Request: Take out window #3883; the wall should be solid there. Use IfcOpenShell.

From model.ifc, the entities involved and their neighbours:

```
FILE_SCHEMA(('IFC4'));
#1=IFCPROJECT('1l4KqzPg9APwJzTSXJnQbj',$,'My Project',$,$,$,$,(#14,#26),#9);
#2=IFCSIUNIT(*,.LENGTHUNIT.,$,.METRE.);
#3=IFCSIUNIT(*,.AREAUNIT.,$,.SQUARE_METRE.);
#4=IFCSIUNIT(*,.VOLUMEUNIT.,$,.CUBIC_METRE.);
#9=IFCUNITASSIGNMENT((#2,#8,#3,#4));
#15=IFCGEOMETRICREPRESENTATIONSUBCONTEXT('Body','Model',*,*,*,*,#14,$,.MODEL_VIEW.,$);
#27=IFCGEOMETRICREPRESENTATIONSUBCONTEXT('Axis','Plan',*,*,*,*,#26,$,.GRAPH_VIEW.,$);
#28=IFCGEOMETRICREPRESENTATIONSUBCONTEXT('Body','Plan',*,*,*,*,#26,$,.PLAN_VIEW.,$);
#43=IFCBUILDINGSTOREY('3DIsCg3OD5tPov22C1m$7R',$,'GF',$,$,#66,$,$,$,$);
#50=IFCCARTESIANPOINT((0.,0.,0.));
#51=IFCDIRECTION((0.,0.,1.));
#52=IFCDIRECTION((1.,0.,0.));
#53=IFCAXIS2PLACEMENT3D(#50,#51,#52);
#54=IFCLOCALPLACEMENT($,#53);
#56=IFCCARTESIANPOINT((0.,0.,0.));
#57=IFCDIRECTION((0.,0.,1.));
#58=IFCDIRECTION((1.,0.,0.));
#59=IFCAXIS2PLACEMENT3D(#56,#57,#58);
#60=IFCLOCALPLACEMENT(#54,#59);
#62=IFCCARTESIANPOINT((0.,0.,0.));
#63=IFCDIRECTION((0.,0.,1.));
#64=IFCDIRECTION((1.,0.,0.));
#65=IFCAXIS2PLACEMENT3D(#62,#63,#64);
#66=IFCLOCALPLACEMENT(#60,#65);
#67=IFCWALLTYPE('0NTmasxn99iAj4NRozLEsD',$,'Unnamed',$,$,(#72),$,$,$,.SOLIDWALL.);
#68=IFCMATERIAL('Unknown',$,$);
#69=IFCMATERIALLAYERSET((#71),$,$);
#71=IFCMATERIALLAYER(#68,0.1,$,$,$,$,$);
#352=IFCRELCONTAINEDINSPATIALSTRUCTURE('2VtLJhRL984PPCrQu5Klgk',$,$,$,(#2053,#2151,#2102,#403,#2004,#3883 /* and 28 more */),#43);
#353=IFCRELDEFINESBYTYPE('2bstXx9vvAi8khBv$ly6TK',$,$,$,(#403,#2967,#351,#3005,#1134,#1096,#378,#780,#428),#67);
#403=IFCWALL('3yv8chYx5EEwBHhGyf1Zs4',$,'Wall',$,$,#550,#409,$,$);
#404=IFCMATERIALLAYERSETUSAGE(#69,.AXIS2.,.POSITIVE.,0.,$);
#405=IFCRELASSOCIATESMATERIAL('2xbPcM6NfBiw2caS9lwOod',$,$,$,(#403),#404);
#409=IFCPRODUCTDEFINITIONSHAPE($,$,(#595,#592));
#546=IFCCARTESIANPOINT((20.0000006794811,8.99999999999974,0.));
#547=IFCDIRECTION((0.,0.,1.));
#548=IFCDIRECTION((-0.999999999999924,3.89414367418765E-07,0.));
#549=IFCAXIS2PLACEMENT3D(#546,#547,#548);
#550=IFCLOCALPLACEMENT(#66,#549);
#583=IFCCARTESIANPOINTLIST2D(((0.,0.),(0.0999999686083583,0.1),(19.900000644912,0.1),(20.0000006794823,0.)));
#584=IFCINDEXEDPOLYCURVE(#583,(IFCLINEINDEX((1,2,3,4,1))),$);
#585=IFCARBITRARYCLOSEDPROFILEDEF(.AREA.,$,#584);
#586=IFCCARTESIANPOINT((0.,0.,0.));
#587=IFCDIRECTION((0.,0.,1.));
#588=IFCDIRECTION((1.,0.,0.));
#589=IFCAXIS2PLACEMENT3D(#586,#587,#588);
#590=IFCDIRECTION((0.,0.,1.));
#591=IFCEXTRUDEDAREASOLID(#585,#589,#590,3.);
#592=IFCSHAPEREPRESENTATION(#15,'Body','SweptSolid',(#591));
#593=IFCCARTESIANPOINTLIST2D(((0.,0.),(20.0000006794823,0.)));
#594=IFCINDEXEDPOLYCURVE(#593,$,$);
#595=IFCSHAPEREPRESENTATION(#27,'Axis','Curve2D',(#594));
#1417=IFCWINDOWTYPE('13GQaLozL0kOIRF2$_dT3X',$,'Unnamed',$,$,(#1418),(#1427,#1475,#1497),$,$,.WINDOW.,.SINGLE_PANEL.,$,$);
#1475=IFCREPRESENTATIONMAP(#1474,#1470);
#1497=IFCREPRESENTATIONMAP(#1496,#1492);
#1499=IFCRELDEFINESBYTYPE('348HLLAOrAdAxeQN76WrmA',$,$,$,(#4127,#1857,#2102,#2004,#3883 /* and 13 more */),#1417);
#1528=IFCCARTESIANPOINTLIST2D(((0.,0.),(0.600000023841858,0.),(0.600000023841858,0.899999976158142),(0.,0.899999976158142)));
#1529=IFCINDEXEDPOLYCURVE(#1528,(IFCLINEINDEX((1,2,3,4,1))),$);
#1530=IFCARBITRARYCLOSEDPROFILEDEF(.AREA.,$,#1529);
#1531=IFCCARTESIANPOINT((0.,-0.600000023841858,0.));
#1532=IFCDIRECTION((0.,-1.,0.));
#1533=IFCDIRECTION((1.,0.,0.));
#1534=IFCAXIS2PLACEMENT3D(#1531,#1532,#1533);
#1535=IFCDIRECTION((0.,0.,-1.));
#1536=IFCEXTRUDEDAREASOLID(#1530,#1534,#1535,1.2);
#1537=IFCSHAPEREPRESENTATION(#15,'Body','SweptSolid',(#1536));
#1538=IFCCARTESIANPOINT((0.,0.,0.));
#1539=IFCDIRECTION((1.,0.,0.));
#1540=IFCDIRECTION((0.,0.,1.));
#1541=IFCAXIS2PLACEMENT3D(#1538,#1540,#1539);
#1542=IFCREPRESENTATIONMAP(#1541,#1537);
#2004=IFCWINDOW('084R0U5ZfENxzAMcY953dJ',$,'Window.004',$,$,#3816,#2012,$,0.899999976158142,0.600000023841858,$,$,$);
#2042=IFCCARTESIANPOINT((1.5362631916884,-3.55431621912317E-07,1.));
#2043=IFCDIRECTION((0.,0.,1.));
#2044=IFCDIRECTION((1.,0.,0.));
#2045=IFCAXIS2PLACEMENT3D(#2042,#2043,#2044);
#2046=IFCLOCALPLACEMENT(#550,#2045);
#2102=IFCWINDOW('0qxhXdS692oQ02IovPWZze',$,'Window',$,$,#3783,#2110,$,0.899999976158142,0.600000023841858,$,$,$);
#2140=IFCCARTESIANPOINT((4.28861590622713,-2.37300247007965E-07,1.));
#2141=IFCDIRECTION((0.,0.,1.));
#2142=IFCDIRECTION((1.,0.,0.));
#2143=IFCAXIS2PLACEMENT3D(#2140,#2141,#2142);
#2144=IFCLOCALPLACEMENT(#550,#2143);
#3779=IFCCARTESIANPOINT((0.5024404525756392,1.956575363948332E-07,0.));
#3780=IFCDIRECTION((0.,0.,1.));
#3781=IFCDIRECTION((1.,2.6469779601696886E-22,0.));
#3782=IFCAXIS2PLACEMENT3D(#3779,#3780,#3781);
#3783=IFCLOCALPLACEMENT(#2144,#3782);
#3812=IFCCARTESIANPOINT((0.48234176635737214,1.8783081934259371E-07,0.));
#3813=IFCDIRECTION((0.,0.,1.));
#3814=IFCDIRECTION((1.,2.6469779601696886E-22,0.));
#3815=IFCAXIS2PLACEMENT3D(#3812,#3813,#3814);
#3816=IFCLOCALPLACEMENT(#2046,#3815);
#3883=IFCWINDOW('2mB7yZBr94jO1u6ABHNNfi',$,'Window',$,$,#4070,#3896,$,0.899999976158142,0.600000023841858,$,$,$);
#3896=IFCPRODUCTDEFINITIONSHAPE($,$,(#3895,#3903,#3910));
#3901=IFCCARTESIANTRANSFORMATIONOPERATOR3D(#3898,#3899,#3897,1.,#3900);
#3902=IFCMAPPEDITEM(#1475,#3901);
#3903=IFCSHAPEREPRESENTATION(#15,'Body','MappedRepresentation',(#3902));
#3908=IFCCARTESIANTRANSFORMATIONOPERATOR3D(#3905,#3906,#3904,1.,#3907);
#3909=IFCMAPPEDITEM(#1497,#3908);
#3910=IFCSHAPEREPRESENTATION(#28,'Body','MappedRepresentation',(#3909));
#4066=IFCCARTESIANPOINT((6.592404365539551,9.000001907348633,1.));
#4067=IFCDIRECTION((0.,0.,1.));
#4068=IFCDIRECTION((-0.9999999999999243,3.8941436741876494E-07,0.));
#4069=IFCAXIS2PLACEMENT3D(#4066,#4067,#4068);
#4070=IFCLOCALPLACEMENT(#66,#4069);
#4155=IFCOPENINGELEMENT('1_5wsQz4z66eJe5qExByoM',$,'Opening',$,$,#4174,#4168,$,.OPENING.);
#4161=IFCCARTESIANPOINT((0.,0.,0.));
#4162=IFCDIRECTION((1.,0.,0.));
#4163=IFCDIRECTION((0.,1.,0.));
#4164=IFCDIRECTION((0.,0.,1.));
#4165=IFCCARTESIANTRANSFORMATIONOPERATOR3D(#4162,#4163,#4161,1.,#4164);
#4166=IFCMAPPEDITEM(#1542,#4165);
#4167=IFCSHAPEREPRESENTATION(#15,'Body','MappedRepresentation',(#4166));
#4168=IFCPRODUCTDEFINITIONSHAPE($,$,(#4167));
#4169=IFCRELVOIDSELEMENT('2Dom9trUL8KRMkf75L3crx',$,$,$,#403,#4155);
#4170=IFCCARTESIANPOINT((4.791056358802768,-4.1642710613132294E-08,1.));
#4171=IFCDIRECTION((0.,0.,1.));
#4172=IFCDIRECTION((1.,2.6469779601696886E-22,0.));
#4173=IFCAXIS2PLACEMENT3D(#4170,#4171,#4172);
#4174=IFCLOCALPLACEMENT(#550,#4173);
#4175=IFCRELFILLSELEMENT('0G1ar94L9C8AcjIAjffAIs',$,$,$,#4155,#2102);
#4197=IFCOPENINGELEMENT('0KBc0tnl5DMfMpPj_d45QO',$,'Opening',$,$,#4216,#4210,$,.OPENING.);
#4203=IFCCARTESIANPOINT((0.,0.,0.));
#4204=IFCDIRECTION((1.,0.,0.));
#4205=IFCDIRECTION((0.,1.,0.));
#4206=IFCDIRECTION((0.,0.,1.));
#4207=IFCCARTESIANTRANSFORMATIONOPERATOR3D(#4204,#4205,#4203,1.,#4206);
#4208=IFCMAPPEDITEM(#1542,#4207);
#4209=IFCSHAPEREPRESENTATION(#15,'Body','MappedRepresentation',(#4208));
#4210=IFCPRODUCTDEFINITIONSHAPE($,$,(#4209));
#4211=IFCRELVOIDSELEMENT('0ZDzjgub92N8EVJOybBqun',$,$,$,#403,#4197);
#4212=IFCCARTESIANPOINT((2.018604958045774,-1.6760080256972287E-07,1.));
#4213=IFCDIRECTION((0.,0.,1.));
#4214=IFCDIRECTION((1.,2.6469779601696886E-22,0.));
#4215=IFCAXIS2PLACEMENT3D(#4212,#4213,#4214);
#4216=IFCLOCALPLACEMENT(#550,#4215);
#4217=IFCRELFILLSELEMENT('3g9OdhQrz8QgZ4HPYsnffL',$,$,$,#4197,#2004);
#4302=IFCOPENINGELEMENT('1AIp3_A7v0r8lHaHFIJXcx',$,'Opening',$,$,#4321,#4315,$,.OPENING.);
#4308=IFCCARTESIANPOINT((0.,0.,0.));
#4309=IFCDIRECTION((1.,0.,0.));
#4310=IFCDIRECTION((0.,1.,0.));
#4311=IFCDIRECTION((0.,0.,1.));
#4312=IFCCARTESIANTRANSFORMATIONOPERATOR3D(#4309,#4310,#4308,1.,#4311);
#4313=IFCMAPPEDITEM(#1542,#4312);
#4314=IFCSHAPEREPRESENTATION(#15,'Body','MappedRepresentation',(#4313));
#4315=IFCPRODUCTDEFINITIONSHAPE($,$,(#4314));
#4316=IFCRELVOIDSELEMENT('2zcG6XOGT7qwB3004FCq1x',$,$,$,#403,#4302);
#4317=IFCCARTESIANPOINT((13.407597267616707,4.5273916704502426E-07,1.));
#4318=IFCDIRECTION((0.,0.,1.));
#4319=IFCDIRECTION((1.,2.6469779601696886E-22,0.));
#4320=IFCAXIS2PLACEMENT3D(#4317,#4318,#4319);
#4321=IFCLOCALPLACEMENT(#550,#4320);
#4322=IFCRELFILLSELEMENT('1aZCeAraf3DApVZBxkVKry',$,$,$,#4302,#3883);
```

```python
import ifcopenshell
import ifcopenshell.api.feature
import ifcopenshell.api.root
import ifcopenshell.geom
import ifcopenshell.util.shape

model = ifcopenshell.open("model.ifc")
settings = ifcopenshell.geom.settings()


def volume(element):
    """Net volume in cubic metres, openings subtracted."""
    shape = ifcopenshell.geom.create_shape(settings, element)
    return ifcopenshell.util.shape.get_volume(shape.geometry)


window = model.by_guid("2mB7yZBr94jO1u6ABHNNfi")
opening = window.FillsVoids[0].RelatingOpeningElement
wall = opening.VoidsElements[0].RelatingBuildingElement
before = volume(wall)

ifcopenshell.api.root.remove_product(model, product=window)
ifcopenshell.api.feature.remove_feature(model, feature=opening)

after = volume(wall)

print(f"wall volume {before:.3f} -> {after:.3f} m3")

model.write("model_updated.ifc")
```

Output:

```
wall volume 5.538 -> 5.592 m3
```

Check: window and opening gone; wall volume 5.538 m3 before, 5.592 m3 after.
